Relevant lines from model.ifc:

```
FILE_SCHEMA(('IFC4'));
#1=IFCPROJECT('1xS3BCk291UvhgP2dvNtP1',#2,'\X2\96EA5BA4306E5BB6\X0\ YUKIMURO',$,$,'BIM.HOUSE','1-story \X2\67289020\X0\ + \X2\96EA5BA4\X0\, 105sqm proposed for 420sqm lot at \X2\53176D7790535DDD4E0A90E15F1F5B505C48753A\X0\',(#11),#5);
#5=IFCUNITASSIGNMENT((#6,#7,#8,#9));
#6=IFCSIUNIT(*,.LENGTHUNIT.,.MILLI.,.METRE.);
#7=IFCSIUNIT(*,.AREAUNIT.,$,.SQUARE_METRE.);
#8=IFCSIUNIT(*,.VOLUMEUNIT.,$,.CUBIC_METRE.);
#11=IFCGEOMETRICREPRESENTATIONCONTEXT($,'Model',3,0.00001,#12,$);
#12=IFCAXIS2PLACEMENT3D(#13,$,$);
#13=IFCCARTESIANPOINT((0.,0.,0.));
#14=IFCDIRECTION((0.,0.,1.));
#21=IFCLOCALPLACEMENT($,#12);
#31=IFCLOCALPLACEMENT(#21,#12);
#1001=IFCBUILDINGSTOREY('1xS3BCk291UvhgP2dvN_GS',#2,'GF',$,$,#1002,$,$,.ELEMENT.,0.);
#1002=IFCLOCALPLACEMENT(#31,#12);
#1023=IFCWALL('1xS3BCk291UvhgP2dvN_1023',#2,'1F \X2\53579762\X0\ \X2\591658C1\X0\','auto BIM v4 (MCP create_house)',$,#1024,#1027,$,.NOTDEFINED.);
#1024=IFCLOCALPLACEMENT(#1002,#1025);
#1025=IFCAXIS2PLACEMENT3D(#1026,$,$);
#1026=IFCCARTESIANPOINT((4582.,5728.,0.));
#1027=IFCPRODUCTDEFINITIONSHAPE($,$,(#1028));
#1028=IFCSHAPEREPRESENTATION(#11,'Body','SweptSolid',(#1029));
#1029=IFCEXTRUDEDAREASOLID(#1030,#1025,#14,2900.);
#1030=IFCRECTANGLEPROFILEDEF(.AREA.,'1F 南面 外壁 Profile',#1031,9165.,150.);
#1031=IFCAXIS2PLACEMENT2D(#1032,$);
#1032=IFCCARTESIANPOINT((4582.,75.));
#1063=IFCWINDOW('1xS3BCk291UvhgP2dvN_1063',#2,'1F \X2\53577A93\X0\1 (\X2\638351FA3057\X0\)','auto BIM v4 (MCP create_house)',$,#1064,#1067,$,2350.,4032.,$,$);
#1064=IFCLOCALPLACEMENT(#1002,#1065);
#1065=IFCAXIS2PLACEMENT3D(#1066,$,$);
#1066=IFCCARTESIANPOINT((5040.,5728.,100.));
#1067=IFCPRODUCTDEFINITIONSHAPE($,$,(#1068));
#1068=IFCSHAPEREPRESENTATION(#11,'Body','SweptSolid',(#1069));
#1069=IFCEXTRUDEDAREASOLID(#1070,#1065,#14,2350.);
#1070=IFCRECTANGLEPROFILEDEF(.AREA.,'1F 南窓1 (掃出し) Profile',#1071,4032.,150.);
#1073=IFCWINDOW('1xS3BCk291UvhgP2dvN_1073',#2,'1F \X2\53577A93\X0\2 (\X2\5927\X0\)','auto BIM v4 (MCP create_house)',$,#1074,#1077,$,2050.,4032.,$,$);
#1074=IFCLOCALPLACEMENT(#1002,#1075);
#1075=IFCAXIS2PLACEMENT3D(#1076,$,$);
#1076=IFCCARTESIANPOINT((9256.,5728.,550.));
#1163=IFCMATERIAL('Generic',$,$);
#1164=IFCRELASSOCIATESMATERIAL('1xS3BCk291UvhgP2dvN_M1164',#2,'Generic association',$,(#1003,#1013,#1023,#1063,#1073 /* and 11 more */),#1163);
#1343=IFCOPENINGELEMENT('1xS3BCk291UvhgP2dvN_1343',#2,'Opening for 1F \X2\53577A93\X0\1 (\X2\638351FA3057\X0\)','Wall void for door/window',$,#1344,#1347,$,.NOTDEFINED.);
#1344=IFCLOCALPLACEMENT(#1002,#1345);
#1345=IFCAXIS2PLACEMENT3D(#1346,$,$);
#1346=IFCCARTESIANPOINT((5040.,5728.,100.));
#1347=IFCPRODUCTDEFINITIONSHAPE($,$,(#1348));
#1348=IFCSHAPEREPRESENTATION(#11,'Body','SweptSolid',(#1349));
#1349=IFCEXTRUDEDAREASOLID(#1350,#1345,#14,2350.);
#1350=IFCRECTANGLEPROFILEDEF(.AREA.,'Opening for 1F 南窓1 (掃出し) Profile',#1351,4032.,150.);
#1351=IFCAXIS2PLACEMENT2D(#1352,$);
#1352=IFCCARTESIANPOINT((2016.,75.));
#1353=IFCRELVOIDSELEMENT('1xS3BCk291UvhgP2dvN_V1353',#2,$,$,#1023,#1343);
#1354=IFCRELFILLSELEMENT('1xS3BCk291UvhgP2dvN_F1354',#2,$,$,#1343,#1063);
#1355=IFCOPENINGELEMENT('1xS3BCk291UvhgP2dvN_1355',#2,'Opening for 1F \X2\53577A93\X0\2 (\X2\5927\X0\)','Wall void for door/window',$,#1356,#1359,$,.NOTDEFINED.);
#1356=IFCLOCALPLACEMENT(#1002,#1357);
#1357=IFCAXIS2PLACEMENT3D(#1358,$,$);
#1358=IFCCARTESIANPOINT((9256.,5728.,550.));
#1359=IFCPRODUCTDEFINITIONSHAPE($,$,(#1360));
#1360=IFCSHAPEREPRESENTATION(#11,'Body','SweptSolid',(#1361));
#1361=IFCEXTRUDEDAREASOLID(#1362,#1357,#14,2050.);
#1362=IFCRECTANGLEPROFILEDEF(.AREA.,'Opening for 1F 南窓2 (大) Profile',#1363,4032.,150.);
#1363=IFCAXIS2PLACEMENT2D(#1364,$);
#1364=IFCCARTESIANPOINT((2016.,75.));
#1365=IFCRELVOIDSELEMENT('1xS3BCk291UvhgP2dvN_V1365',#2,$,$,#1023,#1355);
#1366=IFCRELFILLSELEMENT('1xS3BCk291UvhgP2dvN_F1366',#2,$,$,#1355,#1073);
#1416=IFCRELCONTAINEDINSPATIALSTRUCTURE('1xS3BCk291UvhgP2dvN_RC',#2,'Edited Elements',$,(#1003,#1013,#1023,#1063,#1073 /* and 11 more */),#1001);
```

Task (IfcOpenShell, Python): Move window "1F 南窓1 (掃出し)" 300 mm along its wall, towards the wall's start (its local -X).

```python
import ifcopenshell
import ifcopenshell.api.geometry
import ifcopenshell.util.placement

model = ifcopenshell.open("model.ifc")

window = model.by_id(1063)
opening = window.FillsVoids[0].RelatingOpeningElement
wall = opening.VoidsElements[0].RelatingBuildingElement

wall_matrix = ifcopenshell.util.placement.get_local_placement(wall.ObjectPlacement)
shift = wall_matrix[:3, 0] * -300.0
before = ifcopenshell.util.placement.get_local_placement(window.ObjectPlacement)[:3, 3].copy()

# The window is not placed relative to its opening, so move both.
for product in (opening, window):
    matrix = ifcopenshell.util.placement.get_local_placement(product.ObjectPlacement)
    matrix[:3, 3] += shift
    ifcopenshell.api.geometry.edit_object_placement(model, product=product, matrix=matrix, is_si=False)

after = ifcopenshell.util.placement.get_local_placement(window.ObjectPlacement)[:3, 3]
print("window moved by", (after - before).round(3) + 0.0)

model.write("model_updated.ifc")
```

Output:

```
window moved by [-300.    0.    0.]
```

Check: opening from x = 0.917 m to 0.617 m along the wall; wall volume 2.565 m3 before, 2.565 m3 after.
